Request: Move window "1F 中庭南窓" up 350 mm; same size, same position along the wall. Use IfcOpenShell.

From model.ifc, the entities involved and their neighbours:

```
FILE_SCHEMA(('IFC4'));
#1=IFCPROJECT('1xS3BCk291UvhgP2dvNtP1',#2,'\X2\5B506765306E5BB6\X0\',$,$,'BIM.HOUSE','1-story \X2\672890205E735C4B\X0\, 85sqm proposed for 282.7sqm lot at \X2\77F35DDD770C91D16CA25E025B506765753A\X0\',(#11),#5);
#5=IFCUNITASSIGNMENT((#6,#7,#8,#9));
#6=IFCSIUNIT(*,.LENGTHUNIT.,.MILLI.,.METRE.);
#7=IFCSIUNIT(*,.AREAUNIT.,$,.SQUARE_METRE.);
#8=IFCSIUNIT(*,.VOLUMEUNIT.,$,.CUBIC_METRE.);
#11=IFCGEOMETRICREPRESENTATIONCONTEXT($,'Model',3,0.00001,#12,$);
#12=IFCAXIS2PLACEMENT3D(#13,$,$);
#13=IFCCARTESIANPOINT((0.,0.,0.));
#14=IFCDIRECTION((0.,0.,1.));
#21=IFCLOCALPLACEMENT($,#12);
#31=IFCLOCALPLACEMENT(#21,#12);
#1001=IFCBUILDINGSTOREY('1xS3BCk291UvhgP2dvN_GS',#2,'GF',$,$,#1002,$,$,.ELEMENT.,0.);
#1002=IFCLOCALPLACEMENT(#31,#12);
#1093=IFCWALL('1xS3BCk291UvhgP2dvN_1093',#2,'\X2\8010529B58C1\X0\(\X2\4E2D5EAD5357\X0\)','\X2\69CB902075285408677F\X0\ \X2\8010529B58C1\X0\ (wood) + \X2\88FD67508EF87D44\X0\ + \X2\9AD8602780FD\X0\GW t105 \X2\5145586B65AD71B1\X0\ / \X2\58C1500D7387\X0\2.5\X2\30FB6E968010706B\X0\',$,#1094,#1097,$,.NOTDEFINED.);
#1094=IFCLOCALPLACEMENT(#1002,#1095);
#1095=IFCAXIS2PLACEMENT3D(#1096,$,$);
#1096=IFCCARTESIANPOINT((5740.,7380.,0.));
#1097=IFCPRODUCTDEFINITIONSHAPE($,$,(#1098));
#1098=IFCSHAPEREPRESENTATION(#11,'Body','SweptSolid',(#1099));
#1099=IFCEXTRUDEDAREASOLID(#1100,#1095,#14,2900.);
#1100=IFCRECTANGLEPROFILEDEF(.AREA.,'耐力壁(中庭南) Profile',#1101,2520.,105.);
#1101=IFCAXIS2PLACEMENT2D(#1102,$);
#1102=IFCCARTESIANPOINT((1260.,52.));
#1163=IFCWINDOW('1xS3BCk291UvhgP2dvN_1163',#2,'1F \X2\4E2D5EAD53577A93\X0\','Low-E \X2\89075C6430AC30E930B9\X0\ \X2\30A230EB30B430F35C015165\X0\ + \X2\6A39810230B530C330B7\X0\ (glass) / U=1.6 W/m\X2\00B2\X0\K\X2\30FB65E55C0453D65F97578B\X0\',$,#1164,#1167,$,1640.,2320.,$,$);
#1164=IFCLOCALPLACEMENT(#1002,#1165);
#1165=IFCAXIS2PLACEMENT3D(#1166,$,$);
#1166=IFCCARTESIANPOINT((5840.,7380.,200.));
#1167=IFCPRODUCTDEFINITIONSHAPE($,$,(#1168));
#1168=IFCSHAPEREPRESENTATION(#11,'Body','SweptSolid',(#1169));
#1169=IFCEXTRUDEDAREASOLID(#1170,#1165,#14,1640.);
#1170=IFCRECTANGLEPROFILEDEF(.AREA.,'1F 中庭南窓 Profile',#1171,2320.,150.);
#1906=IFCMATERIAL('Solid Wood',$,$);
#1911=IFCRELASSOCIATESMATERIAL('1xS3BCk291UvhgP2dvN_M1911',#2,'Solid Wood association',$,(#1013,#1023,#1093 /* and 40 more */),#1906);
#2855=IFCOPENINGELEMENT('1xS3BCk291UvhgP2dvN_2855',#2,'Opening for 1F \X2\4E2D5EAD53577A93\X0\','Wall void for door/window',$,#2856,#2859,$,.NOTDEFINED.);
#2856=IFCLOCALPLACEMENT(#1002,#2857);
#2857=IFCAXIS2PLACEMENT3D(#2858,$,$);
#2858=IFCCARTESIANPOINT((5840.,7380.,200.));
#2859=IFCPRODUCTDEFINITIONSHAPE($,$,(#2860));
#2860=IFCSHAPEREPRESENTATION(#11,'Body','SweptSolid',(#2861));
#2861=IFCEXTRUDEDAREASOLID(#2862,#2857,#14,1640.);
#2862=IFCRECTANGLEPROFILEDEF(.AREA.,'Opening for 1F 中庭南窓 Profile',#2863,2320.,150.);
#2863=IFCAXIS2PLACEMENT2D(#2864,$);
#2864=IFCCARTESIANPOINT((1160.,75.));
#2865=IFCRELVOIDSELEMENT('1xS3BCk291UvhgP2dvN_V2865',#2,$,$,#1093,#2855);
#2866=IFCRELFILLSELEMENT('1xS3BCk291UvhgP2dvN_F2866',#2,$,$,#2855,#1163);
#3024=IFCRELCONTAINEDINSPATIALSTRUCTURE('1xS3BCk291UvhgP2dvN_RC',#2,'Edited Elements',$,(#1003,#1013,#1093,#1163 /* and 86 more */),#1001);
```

```python
import numpy as np
import ifcopenshell
import ifcopenshell.api.geometry
import ifcopenshell.util.placement
import ifcopenshell.util.unit

model = ifcopenshell.open("model.ifc")
unit_scale = ifcopenshell.util.unit.calculate_unit_scale(model)

window = model.by_guid("1xS3BCk291UvhgP2dvN_1163")
opening = window.FillsVoids[0].RelatingOpeningElement
dz = 350.0

shift = np.array([0.0, 0.0, dz])
# The window is not placed relative to its opening, so move both.
for product in (opening, window):
    matrix = ifcopenshell.util.placement.get_local_placement(product.ObjectPlacement)
    matrix[:3, 3] += shift
    ifcopenshell.api.geometry.edit_object_placement(model, product=product, matrix=matrix, is_si=False)

print(f"moved by {dz * unit_scale:+.3f} m")

model.write("model_rev.ifc")
```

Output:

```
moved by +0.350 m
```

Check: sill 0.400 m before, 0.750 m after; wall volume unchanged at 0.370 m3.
